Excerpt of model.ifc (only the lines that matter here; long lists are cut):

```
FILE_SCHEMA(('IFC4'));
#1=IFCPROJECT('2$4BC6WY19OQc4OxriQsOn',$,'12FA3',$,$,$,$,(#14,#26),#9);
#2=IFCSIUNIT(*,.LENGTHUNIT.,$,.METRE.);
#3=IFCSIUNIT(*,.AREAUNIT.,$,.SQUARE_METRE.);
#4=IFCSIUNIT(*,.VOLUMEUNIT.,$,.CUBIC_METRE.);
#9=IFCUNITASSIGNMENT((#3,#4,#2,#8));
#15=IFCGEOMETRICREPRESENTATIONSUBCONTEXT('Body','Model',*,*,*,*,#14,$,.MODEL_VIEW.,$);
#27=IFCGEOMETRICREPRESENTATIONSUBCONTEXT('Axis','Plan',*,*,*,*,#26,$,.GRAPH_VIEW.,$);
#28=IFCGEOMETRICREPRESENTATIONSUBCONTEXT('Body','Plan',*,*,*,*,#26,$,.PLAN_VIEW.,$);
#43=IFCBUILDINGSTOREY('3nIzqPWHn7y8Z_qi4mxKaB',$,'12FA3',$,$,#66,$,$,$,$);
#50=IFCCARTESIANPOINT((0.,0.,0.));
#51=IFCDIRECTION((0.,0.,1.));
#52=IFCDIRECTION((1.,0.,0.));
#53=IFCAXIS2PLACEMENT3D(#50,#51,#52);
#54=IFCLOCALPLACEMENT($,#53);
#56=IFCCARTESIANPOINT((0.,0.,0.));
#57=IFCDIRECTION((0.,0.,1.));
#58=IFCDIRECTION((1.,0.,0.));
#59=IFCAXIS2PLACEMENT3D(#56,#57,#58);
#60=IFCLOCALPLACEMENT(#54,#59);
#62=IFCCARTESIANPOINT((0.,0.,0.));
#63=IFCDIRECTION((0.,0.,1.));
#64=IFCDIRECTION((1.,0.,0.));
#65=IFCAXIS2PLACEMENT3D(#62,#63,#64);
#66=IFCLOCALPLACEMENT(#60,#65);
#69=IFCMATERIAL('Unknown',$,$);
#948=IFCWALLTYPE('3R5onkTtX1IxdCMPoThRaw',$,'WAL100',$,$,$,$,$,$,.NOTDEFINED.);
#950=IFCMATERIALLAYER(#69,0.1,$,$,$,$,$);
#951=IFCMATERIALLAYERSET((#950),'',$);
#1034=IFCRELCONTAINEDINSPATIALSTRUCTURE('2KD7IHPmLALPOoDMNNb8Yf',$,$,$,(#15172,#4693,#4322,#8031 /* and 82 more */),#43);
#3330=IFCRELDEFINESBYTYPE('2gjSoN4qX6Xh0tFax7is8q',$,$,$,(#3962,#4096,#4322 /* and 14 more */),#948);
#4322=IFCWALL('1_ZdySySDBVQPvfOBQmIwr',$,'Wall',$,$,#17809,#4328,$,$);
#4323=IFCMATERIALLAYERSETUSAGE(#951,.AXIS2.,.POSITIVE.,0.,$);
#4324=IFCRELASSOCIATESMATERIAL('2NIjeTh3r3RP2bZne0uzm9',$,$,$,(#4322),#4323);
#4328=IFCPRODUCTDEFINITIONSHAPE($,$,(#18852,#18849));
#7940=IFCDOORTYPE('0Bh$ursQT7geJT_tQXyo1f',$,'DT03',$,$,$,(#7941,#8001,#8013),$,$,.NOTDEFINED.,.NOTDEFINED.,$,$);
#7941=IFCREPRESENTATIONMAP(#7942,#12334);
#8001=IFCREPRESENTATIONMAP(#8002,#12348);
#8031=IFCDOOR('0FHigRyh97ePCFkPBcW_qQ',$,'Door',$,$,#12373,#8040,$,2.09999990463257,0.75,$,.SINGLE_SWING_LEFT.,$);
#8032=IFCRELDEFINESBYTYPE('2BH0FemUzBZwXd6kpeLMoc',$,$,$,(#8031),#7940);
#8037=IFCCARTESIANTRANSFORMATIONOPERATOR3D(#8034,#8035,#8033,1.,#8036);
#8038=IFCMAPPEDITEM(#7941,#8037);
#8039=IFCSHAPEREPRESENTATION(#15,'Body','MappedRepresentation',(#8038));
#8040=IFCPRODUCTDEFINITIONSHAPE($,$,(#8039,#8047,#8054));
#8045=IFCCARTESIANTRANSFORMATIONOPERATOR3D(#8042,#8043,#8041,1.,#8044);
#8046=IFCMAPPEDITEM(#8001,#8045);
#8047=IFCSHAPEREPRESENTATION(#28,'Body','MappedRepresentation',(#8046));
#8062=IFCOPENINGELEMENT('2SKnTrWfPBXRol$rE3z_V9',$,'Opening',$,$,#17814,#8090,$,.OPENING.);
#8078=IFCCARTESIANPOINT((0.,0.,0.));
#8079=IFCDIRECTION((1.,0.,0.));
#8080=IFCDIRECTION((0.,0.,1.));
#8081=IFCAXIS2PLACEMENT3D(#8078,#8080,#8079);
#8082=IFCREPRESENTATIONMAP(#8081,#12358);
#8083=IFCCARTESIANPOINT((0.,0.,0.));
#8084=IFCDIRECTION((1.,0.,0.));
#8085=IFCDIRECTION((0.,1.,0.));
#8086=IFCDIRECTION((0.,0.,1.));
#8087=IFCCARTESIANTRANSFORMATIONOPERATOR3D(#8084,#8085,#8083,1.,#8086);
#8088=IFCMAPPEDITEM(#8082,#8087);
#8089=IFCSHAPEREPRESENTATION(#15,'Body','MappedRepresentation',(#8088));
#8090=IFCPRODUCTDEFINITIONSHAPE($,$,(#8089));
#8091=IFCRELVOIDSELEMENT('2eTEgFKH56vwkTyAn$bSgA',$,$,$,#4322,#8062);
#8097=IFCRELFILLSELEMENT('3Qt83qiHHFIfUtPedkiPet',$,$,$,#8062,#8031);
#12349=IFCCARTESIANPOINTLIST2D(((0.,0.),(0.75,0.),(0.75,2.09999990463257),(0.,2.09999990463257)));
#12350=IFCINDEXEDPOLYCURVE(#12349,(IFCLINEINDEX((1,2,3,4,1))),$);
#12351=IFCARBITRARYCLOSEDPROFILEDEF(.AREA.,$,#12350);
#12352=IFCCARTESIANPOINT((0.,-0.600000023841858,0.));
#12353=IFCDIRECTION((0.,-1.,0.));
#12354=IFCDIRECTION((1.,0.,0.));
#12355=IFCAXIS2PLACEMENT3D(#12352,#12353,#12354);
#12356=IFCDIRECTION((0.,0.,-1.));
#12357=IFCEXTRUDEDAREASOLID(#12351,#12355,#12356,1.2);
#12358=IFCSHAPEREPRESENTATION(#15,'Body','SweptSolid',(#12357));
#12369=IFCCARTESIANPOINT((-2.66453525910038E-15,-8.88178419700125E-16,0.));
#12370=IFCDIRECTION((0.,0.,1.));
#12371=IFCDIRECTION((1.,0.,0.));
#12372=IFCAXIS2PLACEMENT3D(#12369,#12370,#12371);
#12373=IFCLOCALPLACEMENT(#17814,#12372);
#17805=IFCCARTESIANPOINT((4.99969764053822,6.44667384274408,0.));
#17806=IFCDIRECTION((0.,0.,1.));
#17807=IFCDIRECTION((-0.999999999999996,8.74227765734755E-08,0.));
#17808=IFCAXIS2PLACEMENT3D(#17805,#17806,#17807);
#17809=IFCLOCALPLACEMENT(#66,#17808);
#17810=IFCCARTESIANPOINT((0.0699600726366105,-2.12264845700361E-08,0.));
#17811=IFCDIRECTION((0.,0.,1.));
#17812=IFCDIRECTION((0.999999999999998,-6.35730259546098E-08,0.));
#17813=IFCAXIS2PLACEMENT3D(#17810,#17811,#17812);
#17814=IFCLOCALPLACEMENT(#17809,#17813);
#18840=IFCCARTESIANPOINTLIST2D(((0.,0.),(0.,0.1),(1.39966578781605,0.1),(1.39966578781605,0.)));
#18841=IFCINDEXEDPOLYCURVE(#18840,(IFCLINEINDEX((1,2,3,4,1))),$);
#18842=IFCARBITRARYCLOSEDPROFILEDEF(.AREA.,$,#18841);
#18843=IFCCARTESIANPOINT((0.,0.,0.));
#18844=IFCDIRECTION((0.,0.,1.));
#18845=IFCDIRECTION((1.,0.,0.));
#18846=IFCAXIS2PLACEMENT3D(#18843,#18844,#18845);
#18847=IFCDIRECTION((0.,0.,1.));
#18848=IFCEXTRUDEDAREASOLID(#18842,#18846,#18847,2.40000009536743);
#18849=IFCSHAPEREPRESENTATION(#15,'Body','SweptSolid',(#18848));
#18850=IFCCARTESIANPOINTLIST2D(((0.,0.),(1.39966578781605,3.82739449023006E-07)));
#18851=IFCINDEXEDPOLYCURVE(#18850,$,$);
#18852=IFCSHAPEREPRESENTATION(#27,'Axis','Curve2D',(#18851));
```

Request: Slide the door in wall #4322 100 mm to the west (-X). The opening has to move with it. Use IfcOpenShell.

```python
import ifcopenshell
import ifcopenshell.api.geometry
import ifcopenshell.util.placement
import ifcopenshell.util.unit

model = ifcopenshell.open("model.ifc")
unit_scale = ifcopenshell.util.unit.calculate_unit_scale(model)

door = model.by_guid("0FHigRyh97ePCFkPBcW_qQ")
opening = door.FillsVoids[0].RelatingOpeningElement
wall = opening.VoidsElements[0].RelatingBuildingElement

wall_matrix = ifcopenshell.util.placement.get_local_placement(wall.ObjectPlacement)
shift = wall_matrix[:3, 0] * 0.1 / unit_scale
before = ifcopenshell.util.placement.get_local_placement(door.ObjectPlacement)[:3, 3].copy()

# The door is placed relative to its opening, so it follows when the opening moves.
matrix = ifcopenshell.util.placement.get_local_placement(opening.ObjectPlacement)
matrix[:3, 3] += shift
ifcopenshell.api.geometry.edit_object_placement(
    model, product=opening, matrix=matrix, is_si=False, should_transform_children=True
)

after = ifcopenshell.util.placement.get_local_placement(door.ObjectPlacement)[:3, 3]
print("door moved by", (after - before).round(3) + 0.0)

model.write("model_edited.ifc")
```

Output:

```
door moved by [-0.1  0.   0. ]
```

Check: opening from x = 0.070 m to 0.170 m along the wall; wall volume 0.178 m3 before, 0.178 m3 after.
